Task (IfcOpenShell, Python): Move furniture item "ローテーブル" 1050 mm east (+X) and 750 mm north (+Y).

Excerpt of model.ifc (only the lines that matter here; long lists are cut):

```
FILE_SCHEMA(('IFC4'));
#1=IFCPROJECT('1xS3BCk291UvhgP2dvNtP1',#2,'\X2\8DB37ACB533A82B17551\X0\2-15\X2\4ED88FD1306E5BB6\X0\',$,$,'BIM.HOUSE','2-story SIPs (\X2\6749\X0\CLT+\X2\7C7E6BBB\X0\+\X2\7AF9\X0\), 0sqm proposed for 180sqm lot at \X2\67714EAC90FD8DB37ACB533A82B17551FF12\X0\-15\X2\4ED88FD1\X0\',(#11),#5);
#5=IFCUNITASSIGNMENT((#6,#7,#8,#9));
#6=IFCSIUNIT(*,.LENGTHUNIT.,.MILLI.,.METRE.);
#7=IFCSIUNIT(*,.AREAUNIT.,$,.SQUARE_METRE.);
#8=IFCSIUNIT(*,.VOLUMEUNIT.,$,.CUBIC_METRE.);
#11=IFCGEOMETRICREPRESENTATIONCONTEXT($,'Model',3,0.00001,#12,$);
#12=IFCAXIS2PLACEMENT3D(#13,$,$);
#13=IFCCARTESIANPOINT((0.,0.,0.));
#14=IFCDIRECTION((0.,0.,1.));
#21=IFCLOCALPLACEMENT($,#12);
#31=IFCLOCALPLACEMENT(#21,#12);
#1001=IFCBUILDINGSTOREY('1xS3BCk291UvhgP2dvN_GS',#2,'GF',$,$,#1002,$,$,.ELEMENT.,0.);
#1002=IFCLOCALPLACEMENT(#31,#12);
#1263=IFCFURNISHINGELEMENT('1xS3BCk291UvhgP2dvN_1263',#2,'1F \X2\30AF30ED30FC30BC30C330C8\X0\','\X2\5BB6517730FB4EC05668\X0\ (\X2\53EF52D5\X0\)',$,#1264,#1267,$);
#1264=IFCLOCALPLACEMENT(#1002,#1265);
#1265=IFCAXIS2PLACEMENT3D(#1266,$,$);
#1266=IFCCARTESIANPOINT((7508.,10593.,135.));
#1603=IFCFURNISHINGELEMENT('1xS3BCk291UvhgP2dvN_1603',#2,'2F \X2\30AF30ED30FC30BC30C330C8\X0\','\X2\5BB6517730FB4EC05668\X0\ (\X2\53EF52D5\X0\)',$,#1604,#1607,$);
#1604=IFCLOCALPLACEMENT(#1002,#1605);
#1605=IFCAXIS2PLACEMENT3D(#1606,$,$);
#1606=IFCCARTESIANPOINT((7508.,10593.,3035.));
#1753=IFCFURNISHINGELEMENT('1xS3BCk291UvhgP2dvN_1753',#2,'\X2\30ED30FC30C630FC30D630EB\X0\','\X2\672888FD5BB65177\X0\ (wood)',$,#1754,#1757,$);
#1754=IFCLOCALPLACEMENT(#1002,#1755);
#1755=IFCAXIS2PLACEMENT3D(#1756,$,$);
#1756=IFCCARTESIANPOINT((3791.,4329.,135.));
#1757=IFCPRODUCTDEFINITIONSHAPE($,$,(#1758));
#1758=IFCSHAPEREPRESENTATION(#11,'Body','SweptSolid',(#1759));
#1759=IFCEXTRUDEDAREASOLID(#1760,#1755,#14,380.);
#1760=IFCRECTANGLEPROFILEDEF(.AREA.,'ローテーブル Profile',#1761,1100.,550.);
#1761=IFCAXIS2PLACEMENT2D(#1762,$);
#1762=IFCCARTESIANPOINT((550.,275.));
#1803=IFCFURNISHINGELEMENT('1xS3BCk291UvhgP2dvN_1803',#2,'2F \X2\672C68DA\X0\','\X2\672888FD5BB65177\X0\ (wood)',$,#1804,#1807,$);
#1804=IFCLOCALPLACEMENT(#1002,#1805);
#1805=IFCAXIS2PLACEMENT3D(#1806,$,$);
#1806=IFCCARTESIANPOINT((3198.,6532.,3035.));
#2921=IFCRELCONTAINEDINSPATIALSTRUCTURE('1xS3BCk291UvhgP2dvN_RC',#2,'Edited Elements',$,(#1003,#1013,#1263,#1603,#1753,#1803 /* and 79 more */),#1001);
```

```python
import ifcopenshell
import ifcopenshell.api.geometry
import ifcopenshell.util.placement
import ifcopenshell.util.unit

model = ifcopenshell.open("model.ifc")
unit_scale = ifcopenshell.util.unit.calculate_unit_scale(model)

item = model.by_guid("1xS3BCk291UvhgP2dvN_1753")
matrix = ifcopenshell.util.placement.get_local_placement(item.ObjectPlacement)
matrix[0, 3] += 1.05 / unit_scale
matrix[1, 3] += 0.75 / unit_scale
ifcopenshell.api.geometry.edit_object_placement(model, product=item, matrix=matrix, is_si=False)

print(ifcopenshell.util.placement.get_local_placement(item.ObjectPlacement).round(3) + 0.0)

model.write("model-out.ifc")
```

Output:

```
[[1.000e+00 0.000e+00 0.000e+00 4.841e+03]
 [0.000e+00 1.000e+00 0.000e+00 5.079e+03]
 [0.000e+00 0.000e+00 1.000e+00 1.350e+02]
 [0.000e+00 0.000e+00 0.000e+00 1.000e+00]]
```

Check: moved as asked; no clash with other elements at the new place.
